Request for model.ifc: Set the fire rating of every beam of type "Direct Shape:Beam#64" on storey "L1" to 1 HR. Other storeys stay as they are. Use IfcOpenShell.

First a look at what the model holds.

```python
import ifcopenshell
import ifcopenshell.util.element

model = ifcopenshell.open("model.ifc")
print(model.schema)
storey = next(s for s in model.by_type("IfcBuildingStorey") if s.Name == "L1")
beams = [e for e in ifcopenshell.util.element.get_decomposition(storey) if e.is_a("IfcBeam")]
seen = {}
for e in beams:
    element_type = ifcopenshell.util.element.get_type(e)
    key = (element_type.Name if element_type != e and element_type else None, ifcopenshell.util.element.get_pset(e, "Pset_BeamCommon", "FireRating"))
    seen[key] = seen.get(key, 0) + 1
for (name, value), count in sorted(seen.items(), key=str):
    print(count, "x", name, "|", value)
```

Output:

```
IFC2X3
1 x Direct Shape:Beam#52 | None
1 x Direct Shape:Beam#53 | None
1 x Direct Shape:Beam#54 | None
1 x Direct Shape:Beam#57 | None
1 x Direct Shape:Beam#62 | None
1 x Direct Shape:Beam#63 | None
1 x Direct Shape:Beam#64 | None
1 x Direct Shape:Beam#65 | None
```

```python
import ifcopenshell
import ifcopenshell.api.pset
import ifcopenshell.util.element

model = ifcopenshell.open("model.ifc")

storey = next(s for s in model.by_type("IfcBuildingStorey") if s.Name == "L1")
beams = [e for e in ifcopenshell.util.element.get_decomposition(storey) if e.is_a("IfcBeam")]

count = 0
for e in beams:
    element_type = ifcopenshell.util.element.get_type(e)
    if element_type in (None, e) or element_type.Name != "Direct Shape:Beam#64":
        continue
    # add_pset returns the element's existing set when there is one.
    pset = ifcopenshell.api.pset.add_pset(model, product=e, name="Pset_BeamCommon")
    ifcopenshell.api.pset.edit_pset(model, pset=pset, properties={"FireRating": "1 HR"})
    count += 1

print(count, "beams updated")

model.write("model_v2.ifc")
```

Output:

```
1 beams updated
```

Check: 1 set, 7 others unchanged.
